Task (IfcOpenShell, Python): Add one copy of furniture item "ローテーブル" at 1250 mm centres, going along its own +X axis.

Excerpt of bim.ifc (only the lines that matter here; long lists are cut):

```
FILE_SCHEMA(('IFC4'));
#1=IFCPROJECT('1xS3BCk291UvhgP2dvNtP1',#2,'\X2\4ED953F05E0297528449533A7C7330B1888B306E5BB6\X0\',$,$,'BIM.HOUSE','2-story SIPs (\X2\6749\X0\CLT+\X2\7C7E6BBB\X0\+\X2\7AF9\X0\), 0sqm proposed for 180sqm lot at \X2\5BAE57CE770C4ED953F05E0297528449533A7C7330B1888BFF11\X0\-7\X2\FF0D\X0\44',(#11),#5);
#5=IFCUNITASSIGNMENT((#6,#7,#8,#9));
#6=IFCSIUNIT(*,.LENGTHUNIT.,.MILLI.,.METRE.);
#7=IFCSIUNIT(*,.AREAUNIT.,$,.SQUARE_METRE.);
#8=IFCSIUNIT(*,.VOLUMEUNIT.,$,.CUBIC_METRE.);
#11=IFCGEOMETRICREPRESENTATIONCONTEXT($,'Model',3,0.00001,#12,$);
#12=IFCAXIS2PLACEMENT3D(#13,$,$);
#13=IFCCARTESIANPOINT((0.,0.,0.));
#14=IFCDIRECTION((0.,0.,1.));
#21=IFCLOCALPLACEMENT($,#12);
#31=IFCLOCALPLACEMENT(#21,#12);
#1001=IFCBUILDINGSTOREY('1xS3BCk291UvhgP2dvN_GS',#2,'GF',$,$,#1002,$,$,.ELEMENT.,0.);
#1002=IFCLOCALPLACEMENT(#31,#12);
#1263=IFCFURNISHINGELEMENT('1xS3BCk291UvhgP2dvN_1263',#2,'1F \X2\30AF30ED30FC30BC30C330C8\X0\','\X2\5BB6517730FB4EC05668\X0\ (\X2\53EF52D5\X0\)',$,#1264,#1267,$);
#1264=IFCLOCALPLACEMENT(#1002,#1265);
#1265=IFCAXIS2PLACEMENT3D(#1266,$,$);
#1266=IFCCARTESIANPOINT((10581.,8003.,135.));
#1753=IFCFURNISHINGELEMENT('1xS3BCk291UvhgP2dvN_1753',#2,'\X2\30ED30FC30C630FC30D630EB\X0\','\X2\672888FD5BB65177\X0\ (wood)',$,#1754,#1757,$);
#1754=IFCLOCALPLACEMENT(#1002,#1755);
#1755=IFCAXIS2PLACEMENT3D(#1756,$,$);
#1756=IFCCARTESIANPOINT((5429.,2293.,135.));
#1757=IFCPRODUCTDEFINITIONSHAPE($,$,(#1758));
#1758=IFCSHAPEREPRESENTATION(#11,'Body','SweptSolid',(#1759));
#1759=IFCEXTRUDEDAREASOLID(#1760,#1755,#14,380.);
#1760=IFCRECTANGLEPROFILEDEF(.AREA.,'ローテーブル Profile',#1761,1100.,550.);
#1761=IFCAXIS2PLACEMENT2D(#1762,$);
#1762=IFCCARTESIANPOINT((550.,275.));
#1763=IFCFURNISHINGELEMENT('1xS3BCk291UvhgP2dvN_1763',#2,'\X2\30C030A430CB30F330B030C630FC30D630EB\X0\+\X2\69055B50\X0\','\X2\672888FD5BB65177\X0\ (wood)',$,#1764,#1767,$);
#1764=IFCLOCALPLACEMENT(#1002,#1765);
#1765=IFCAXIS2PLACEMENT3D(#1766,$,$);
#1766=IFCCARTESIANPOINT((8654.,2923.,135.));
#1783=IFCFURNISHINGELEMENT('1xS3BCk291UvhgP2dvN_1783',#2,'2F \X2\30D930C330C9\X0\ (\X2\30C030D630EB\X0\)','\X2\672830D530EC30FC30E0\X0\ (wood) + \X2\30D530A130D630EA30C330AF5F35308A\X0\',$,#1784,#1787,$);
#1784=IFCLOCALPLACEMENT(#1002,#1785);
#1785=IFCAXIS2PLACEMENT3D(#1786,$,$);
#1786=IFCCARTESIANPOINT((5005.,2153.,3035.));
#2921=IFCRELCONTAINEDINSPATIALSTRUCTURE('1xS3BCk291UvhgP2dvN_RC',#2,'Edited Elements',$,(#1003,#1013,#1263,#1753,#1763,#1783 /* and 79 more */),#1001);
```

```python
import ifcopenshell
import ifcopenshell.api.geometry
import ifcopenshell.api.root
import ifcopenshell.util.element
import ifcopenshell.util.placement

model = ifcopenshell.open("bim.ifc")


def reuse_history(source, copy):
    """copy_class also copies each property set's owner history, people and application; keep the originals."""
    for rel in copy.IsDefinedBy:
        if rel.is_a("IfcRelDefinesByProperties") and (history := rel.RelatingPropertyDefinition.OwnerHistory):
            rel.RelatingPropertyDefinition.OwnerHistory = source.OwnerHistory
            ifcopenshell.util.element.remove_deep2(model, history)


source = model.by_id(1753)
base = ifcopenshell.util.placement.get_local_placement(source.ObjectPlacement)
step = base[:3, 0] * 1250.0

for i in range(1, 2):
    copy = ifcopenshell.api.root.copy_class(model, product=source)
    copy.Representation = ifcopenshell.util.element.copy_deep(
        model, source.Representation, exclude=["IfcGeometricRepresentationContext", "IfcRepresentationMap"]
    )
    reuse_history(source, copy)
    matrix = base.copy()
    matrix[:3, 3] += i * step
    print("added at", matrix[:3, 3].round(3) + 0.0)
    ifcopenshell.api.geometry.edit_object_placement(model, product=copy, matrix=matrix, is_si=False)

model.write("bim_updated.ifc")
```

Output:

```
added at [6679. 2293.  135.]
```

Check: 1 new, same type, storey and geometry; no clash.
